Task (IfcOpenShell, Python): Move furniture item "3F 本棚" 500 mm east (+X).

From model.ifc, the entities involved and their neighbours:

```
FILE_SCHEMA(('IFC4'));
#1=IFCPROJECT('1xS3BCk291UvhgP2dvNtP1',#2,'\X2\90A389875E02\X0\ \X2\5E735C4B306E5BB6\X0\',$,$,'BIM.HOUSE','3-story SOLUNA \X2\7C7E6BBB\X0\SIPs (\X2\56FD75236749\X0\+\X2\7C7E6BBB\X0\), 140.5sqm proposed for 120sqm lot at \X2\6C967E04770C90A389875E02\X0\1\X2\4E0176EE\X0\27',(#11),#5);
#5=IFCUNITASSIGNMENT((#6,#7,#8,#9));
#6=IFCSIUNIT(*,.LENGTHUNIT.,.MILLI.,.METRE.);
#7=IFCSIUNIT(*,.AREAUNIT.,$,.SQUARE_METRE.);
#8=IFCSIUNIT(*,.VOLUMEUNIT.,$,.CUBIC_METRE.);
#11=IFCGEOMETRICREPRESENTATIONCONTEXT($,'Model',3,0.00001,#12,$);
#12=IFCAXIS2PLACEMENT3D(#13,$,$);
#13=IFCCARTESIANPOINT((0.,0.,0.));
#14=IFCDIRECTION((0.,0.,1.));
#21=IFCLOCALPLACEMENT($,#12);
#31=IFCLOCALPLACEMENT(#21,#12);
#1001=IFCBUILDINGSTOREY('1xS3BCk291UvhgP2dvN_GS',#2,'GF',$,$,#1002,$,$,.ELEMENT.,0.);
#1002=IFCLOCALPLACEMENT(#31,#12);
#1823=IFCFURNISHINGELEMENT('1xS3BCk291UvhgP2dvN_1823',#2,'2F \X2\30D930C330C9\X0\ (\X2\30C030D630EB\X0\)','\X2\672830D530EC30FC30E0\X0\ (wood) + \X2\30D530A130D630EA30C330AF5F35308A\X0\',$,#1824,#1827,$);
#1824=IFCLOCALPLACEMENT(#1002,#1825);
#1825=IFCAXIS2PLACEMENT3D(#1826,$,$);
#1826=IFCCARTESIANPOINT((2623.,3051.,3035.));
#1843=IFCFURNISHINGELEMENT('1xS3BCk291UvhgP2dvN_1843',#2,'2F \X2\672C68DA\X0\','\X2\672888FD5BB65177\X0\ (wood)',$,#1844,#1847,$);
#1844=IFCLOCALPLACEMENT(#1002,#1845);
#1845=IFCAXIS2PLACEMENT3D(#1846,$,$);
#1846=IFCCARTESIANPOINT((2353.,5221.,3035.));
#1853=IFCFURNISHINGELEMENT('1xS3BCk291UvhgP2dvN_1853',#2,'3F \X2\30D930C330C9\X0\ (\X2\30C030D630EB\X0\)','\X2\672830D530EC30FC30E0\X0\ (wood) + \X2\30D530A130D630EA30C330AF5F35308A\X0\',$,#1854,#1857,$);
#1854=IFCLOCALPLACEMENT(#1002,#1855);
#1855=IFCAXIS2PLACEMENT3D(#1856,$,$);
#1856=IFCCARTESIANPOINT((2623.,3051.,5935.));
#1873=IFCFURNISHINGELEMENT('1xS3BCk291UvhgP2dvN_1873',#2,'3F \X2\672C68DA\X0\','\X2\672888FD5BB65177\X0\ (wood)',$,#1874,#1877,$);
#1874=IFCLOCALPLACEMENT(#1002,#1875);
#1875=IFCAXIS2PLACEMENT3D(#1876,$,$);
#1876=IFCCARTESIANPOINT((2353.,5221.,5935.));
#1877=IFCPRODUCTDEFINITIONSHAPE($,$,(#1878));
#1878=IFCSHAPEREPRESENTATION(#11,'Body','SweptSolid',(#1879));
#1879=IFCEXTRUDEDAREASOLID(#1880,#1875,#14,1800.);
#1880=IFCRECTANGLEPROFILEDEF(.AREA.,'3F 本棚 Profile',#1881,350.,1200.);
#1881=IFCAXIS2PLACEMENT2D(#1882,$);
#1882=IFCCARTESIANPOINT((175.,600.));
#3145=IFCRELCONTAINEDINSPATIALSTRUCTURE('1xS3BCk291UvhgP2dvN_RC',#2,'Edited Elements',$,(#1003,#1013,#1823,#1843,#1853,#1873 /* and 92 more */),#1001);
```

```python
import ifcopenshell
import ifcopenshell.api.geometry
import ifcopenshell.util.placement
import ifcopenshell.util.unit

model = ifcopenshell.open("model.ifc")
unit_scale = ifcopenshell.util.unit.calculate_unit_scale(model)

item = model.by_id(1873)
matrix = ifcopenshell.util.placement.get_local_placement(item.ObjectPlacement)
matrix[0, 3] += 0.5 / unit_scale
ifcopenshell.api.geometry.edit_object_placement(model, product=item, matrix=matrix, is_si=False)

print(ifcopenshell.util.placement.get_local_placement(item.ObjectPlacement).round(3) + 0.0)

model.write("model-out.ifc")
```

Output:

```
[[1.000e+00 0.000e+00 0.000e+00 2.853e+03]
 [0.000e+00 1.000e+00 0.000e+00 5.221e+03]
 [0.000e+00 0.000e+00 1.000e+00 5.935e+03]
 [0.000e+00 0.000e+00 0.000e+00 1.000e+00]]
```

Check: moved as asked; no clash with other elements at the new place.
